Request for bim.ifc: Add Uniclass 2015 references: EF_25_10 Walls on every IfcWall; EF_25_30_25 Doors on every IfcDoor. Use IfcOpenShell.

First a look at what the model holds.

```python
import ifcopenshell

model = ifcopenshell.open("bim.ifc")
print(model.schema)
print("classifications:", [c.Name for c in model.by_type("IfcClassification")])
for ifc_class in ("IfcDoor", "IfcRoof", "IfcStair", "IfcWall", "IfcWindow"):
    print(ifc_class, len(model.by_type(ifc_class)))
```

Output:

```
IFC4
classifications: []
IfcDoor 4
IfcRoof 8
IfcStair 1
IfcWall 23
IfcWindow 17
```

```python
import ifcopenshell
import ifcopenshell.api.classification

model = ifcopenshell.open("bim.ifc")

system = ifcopenshell.api.classification.add_classification(model, classification="Uniclass 2015")

codes = {
    "IfcWall": ("EF_25_10", "Walls"),
    "IfcDoor": ("EF_25_30_25", "Doors"),
}
for ifc_class, (code, name) in codes.items():
    products = model.by_type(ifc_class)
    ifcopenshell.api.classification.add_reference(
        model, products=products, classification=system, identification=code, name=name
    )
    print(code, len(products))

model.write("bim_v2.ifc")
```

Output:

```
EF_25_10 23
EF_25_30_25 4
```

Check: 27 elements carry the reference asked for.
